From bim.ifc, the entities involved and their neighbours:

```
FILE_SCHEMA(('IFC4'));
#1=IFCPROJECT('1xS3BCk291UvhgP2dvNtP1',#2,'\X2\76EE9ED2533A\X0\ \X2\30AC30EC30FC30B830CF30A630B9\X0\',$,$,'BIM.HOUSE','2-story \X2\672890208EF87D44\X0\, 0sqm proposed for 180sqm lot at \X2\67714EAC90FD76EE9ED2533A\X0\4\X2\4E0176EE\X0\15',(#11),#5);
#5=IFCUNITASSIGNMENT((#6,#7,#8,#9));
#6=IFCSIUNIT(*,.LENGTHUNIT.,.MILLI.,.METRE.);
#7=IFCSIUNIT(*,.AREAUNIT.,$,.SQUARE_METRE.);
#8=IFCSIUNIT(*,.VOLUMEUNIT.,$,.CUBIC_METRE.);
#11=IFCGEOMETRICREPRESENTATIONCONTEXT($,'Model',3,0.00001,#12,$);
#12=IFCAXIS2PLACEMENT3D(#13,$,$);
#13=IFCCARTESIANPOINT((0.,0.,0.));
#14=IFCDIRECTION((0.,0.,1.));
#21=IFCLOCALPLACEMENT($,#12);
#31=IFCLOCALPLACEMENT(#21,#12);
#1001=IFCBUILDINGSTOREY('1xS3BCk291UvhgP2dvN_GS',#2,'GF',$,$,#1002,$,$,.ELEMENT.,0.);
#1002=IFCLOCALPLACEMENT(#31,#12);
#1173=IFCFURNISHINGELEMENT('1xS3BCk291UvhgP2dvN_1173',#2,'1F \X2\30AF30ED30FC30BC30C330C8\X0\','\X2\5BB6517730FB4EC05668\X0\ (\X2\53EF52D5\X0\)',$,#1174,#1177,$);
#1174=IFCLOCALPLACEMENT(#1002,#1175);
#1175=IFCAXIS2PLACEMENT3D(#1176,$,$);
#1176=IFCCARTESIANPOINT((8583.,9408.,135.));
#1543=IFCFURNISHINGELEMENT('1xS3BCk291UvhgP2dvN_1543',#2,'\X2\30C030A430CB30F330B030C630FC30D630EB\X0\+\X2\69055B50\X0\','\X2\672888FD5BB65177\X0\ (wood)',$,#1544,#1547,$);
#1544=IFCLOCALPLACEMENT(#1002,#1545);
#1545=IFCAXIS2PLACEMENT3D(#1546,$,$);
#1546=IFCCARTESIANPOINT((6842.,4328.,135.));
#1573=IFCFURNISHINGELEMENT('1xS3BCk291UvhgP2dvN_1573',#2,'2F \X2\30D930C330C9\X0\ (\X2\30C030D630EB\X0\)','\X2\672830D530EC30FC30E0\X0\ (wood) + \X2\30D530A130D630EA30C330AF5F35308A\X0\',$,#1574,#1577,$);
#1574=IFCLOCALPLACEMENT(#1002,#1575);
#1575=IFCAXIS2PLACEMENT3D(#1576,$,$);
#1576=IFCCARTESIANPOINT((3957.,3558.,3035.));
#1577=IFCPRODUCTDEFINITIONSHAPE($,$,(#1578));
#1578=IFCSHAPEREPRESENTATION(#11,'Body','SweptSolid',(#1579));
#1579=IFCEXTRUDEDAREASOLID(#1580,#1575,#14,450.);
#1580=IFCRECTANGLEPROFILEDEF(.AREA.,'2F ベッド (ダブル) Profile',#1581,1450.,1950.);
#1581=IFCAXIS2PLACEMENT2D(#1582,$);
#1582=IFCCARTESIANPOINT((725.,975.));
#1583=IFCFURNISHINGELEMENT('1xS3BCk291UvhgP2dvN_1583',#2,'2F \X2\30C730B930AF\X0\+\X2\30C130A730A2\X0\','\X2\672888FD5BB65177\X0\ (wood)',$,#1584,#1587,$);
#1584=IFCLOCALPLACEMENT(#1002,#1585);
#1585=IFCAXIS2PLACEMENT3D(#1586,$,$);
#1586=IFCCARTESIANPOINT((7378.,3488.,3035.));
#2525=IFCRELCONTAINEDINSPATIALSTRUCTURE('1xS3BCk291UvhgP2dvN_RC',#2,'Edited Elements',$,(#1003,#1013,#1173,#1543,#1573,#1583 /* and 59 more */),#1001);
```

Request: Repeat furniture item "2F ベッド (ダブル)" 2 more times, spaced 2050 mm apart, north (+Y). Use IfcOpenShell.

```python
import numpy as np
import ifcopenshell
import ifcopenshell.api.geometry
import ifcopenshell.api.root
import ifcopenshell.util.element
import ifcopenshell.util.placement

model = ifcopenshell.open("bim.ifc")


def reuse_history(source, copy):
    """copy_class also copies each property set's owner history, people and application; keep the originals."""
    for rel in copy.IsDefinedBy:
        if rel.is_a("IfcRelDefinesByProperties") and (history := rel.RelatingPropertyDefinition.OwnerHistory):
            rel.RelatingPropertyDefinition.OwnerHistory = source.OwnerHistory
            ifcopenshell.util.element.remove_deep2(model, history)


source = model.by_guid("1xS3BCk291UvhgP2dvN_1573")
base = ifcopenshell.util.placement.get_local_placement(source.ObjectPlacement)
step = np.array([0.0, 1.0, 0.0]) * 2050.0

for i in range(1, 3):
    copy = ifcopenshell.api.root.copy_class(model, product=source)
    copy.Representation = ifcopenshell.util.element.copy_deep(
        model, source.Representation, exclude=["IfcGeometricRepresentationContext", "IfcRepresentationMap"]
    )
    reuse_history(source, copy)
    matrix = base.copy()
    matrix[:3, 3] += i * step
    print("added at", matrix[:3, 3].round(3) + 0.0)
    ifcopenshell.api.geometry.edit_object_placement(model, product=copy, matrix=matrix, is_si=False)

model.write("bim_rev.ifc")
```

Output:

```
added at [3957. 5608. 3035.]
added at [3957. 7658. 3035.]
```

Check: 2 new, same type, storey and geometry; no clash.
